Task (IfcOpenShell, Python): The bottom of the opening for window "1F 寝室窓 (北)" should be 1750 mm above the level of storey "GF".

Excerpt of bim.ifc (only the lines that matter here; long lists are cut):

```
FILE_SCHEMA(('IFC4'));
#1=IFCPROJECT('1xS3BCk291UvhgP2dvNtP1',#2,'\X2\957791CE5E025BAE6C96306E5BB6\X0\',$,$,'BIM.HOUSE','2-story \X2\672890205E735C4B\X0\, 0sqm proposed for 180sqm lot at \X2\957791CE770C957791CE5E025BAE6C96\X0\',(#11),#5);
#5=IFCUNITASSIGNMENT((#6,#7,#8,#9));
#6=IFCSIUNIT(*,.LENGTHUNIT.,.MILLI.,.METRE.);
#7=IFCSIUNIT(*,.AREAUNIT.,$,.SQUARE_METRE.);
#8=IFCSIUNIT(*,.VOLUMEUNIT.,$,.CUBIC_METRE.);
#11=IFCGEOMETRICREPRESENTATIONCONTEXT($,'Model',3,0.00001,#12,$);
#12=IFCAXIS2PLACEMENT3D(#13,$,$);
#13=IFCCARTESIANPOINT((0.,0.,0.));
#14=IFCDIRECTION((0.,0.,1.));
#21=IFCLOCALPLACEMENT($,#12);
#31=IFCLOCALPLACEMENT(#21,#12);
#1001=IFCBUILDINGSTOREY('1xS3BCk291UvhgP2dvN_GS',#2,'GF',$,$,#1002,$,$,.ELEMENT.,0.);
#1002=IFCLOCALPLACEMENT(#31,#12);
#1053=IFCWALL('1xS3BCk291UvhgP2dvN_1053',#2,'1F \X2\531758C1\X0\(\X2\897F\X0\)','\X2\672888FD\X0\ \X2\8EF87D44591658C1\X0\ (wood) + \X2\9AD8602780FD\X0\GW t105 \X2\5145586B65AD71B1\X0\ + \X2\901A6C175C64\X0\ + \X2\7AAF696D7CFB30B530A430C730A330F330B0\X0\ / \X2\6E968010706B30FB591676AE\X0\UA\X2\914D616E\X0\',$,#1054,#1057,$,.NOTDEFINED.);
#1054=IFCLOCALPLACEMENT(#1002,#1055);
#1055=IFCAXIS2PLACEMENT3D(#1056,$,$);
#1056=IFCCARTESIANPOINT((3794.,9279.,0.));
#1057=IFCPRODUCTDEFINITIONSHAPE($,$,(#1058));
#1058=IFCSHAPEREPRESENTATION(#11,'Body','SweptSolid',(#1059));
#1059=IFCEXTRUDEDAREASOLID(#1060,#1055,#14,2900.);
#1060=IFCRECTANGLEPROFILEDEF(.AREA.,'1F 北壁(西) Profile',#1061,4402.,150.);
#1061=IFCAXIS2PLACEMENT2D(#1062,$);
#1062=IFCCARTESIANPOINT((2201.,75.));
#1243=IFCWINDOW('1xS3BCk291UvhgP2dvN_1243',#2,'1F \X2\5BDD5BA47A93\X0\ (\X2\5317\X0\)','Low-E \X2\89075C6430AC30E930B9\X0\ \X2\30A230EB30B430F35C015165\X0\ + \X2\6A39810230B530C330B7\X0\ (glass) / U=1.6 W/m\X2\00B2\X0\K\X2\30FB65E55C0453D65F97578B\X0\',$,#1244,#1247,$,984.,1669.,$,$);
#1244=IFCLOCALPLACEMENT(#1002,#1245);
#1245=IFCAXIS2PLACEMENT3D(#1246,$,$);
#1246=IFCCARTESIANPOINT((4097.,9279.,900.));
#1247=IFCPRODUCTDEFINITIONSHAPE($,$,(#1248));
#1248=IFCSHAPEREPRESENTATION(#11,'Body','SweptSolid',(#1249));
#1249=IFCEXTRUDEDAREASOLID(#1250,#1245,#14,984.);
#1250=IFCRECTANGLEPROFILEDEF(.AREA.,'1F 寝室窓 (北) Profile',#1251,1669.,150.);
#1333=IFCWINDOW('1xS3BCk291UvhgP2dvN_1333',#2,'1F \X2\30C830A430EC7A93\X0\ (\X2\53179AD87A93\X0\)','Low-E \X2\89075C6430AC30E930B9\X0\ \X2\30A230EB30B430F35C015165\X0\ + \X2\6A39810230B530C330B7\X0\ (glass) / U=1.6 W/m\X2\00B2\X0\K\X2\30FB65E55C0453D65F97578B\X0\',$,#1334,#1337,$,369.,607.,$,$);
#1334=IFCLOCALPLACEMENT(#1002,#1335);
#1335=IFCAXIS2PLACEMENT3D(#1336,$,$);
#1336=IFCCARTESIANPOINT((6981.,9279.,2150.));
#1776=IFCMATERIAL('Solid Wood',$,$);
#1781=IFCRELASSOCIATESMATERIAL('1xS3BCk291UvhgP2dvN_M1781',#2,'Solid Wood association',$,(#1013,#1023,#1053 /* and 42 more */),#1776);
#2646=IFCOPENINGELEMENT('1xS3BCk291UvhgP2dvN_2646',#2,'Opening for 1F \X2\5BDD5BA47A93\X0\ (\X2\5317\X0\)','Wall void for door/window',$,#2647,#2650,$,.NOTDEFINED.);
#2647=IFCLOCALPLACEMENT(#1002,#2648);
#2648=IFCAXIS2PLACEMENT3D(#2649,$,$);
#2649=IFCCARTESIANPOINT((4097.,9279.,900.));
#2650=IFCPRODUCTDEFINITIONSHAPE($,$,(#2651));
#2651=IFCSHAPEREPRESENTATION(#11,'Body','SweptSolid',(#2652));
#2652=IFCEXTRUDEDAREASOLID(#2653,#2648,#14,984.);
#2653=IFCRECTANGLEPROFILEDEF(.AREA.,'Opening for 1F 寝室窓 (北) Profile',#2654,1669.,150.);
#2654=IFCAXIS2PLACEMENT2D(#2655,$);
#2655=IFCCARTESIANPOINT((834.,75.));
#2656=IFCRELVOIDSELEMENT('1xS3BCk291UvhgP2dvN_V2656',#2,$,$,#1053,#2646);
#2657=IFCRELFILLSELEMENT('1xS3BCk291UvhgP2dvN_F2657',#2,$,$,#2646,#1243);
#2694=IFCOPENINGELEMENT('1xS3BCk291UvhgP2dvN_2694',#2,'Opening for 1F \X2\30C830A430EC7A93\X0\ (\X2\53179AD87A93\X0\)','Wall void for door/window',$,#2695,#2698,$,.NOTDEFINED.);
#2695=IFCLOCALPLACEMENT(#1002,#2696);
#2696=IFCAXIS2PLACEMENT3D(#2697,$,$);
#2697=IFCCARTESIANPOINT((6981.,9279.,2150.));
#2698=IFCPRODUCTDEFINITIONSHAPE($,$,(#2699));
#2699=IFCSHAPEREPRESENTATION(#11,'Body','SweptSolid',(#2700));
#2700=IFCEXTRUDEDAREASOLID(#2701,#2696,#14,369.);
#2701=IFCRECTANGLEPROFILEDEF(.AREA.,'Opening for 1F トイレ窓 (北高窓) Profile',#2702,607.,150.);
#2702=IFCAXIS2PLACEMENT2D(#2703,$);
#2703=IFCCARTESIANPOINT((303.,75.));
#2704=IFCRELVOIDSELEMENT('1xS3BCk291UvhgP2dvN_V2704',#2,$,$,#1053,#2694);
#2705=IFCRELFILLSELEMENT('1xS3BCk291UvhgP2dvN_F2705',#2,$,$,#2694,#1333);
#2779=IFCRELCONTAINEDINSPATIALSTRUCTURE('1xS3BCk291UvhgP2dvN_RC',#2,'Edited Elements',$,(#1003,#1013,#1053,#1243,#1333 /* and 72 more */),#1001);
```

```python
import numpy as np
import ifcopenshell
import ifcopenshell.api.geometry
import ifcopenshell.geom
import ifcopenshell.util.element
import ifcopenshell.util.placement
import ifcopenshell.util.shape
import ifcopenshell.util.unit

model = ifcopenshell.open("bim.ifc")
unit_scale = ifcopenshell.util.unit.calculate_unit_scale(model)

window = model.by_id(1243)
opening = window.FillsVoids[0].RelatingOpeningElement
storey = ifcopenshell.util.element.get_container(window, ifc_class="IfcBuildingStorey")
level = ifcopenshell.util.placement.get_local_placement(storey.ObjectPlacement)[2, 3]

# The opening's origin need not be at the sill, so measure its lowest point.
shape = ifcopenshell.geom.create_shape(ifcopenshell.geom.settings(), opening)
bottom = ifcopenshell.util.shape.get_shape_bottom_elevation(shape, shape.geometry) / unit_scale
dz = level + 1.75 / unit_scale - bottom

shift = np.array([0.0, 0.0, dz])
# The window is not placed relative to its opening, so move both.
for product in (opening, window):
    matrix = ifcopenshell.util.placement.get_local_placement(product.ObjectPlacement)
    matrix[:3, 3] += shift
    ifcopenshell.api.geometry.edit_object_placement(model, product=product, matrix=matrix, is_si=False)

print(f"moved by {dz * unit_scale:+.3f} m")

model.write("bim-out.ifc")
```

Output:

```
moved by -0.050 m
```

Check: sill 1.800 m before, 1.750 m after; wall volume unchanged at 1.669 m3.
